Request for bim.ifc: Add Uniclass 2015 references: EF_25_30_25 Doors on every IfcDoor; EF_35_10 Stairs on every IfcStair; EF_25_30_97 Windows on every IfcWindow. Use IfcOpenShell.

First a look at what the model holds.

```python
import ifcopenshell

model = ifcopenshell.open("bim.ifc")
print(model.schema)
print("classifications:", [c.Name for c in model.by_type("IfcClassification")])
for ifc_class in ("IfcDoor", "IfcRoof", "IfcStair", "IfcWall", "IfcWindow"):
    print(ifc_class, len(model.by_type(ifc_class)))
```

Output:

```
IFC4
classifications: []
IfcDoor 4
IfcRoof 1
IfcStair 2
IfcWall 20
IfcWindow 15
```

```python
import ifcopenshell
import ifcopenshell.api.classification

model = ifcopenshell.open("bim.ifc")

system = ifcopenshell.api.classification.add_classification(model, classification="Uniclass 2015")

codes = {
    "IfcDoor": ("EF_25_30_25", "Doors"),
    "IfcStair": ("EF_35_10", "Stairs"),
    "IfcWindow": ("EF_25_30_97", "Windows"),
}
for ifc_class, (code, name) in codes.items():
    products = model.by_type(ifc_class)
    ifcopenshell.api.classification.add_reference(
        model, products=products, classification=system, identification=code, name=name
    )
    print(code, len(products))

model.write("bim_edited.ifc")
```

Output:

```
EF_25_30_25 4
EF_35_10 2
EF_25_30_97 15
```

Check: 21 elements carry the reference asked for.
